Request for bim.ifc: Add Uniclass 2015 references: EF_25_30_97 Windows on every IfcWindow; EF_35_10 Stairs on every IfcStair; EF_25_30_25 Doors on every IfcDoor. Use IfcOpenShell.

First a look at what the model holds.

```python
import ifcopenshell

model = ifcopenshell.open("bim.ifc")
print(model.schema)
print("classifications:", [c.Name for c in model.by_type("IfcClassification")])
for ifc_class in ("IfcDoor", "IfcRoof", "IfcStair", "IfcWall", "IfcWindow"):
    print(ifc_class, len(model.by_type(ifc_class)))
```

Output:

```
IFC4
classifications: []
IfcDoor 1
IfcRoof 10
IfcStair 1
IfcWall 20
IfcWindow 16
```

```python
import ifcopenshell
import ifcopenshell.api.classification

model = ifcopenshell.open("bim.ifc")

system = ifcopenshell.api.classification.add_classification(model, classification="Uniclass 2015")

codes = {
    "IfcWindow": ("EF_25_30_97", "Windows"),
    "IfcStair": ("EF_35_10", "Stairs"),
    "IfcDoor": ("EF_25_30_25", "Doors"),
}
for ifc_class, (code, name) in codes.items():
    products = model.by_type(ifc_class)
    ifcopenshell.api.classification.add_reference(
        model, products=products, classification=system, identification=code, name=name
    )
    print(code, len(products))

model.write("bim_v2.ifc")
```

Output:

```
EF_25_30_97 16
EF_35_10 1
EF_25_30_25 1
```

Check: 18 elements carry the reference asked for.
